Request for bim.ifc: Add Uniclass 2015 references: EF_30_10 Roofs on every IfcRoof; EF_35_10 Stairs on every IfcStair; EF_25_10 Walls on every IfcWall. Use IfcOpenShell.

First a look at what the model holds.

```python
import ifcopenshell

model = ifcopenshell.open("bim.ifc")
print(model.schema)
print("classifications:", [c.Name for c in model.by_type("IfcClassification")])
for ifc_class in ("IfcDoor", "IfcRoof", "IfcStair", "IfcWall", "IfcWindow"):
    print(ifc_class, len(model.by_type(ifc_class)))
```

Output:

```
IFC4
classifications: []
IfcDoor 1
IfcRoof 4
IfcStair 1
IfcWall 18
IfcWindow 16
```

```python
import ifcopenshell
import ifcopenshell.api.classification

model = ifcopenshell.open("bim.ifc")

system = ifcopenshell.api.classification.add_classification(model, classification="Uniclass 2015")

codes = {
    "IfcRoof": ("EF_30_10", "Roofs"),
    "IfcStair": ("EF_35_10", "Stairs"),
    "IfcWall": ("EF_25_10", "Walls"),
}
for ifc_class, (code, name) in codes.items():
    products = model.by_type(ifc_class)
    ifcopenshell.api.classification.add_reference(
        model, products=products, classification=system, identification=code, name=name
    )
    print(code, len(products))

model.write("bim_v2.ifc")
```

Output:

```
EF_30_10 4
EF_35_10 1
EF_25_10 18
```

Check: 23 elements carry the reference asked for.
